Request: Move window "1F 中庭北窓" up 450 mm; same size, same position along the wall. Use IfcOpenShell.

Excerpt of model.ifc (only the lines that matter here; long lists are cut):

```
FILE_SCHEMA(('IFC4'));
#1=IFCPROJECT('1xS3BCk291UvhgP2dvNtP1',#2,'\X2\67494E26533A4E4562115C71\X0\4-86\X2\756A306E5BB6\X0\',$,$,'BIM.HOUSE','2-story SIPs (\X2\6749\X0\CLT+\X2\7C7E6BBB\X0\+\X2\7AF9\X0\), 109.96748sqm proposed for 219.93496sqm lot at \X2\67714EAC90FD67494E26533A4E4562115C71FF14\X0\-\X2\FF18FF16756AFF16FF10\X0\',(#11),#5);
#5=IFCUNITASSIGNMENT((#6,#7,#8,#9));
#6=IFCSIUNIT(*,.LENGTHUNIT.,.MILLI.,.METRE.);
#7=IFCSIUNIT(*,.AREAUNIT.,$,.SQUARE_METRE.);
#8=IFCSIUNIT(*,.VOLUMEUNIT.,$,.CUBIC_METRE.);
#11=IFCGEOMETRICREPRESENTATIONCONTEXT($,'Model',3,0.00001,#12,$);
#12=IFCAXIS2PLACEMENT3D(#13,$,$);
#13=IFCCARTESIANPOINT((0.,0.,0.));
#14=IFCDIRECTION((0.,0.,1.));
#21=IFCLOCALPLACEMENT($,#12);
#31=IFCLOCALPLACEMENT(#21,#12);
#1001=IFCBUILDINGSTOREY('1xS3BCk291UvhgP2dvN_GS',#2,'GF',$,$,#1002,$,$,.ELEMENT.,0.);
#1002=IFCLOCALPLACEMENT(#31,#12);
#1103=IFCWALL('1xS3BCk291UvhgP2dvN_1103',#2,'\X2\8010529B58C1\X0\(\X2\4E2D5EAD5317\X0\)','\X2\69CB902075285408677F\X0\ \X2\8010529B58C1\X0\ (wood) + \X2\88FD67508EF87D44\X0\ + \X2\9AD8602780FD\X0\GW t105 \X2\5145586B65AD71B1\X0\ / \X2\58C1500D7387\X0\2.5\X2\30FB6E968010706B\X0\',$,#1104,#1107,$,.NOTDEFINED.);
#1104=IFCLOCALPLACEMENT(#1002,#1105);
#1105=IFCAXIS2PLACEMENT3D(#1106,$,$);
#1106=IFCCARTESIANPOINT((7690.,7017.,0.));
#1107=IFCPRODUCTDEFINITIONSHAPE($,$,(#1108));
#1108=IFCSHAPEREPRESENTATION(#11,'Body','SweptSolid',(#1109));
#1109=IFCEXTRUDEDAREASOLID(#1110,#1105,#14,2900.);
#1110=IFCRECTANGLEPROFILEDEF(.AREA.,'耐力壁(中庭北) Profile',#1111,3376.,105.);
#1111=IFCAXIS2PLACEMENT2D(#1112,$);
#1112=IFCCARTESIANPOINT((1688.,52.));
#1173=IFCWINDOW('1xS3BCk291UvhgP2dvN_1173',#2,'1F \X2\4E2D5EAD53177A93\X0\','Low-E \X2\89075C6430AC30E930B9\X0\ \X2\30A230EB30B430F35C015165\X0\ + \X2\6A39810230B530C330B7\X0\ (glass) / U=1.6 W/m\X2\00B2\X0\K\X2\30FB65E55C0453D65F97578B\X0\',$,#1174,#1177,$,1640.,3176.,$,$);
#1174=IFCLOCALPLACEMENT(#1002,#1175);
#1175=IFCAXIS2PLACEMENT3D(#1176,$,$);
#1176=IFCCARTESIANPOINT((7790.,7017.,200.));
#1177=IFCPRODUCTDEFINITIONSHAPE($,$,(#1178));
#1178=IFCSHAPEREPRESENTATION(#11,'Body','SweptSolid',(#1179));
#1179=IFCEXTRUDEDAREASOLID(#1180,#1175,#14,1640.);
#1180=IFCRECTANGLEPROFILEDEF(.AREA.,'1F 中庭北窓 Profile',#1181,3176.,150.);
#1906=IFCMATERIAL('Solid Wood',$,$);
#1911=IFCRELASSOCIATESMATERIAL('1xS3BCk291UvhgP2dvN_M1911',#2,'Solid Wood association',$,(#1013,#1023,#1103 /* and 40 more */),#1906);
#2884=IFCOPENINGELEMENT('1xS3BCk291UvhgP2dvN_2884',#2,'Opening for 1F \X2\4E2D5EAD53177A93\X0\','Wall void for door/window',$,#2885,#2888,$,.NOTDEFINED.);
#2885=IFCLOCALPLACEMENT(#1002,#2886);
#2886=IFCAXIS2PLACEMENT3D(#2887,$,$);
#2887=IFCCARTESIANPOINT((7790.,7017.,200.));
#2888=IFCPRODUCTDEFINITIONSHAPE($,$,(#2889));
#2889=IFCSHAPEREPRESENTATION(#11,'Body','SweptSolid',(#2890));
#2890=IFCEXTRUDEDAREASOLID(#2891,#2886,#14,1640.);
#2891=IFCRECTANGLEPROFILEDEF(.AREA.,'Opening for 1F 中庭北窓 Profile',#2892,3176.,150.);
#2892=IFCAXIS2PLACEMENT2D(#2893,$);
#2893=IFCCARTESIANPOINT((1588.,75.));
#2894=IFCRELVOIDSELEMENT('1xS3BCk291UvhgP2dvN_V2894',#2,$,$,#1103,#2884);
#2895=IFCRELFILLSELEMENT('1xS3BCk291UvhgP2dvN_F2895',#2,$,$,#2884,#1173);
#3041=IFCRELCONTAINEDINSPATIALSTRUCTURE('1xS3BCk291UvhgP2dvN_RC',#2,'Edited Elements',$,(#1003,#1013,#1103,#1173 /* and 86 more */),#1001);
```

```python
import numpy as np
import ifcopenshell
import ifcopenshell.api.geometry
import ifcopenshell.util.placement
import ifcopenshell.util.unit

model = ifcopenshell.open("model.ifc")
unit_scale = ifcopenshell.util.unit.calculate_unit_scale(model)

window = model.by_id(1173)
opening = window.FillsVoids[0].RelatingOpeningElement
dz = 0.45 / unit_scale

shift = np.array([0.0, 0.0, dz])
# The window is not placed relative to its opening, so move both.
for product in (opening, window):
    matrix = ifcopenshell.util.placement.get_local_placement(product.ObjectPlacement)
    matrix[:3, 3] += shift
    ifcopenshell.api.geometry.edit_object_placement(model, product=product, matrix=matrix, is_si=False)

print(f"moved by {dz * unit_scale:+.3f} m")

model.write("model_updated.ifc")
```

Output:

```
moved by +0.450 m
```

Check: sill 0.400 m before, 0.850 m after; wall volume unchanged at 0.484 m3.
